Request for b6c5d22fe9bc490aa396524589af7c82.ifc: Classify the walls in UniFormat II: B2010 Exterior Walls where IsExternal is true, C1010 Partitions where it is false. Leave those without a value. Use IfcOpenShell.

First a look at what the model holds.

```python
import ifcopenshell
import ifcopenshell.util.element

model = ifcopenshell.open("b6c5d22fe9bc490aa396524589af7c82.ifc")
print(model.schema)
print("classifications:", [c.Name for c in model.by_type("IfcClassification")])
values = [ifcopenshell.util.element.get_pset(e, "Pset_WallCommon", "IsExternal") for e in model.by_type("IfcWall")]
for value in (True, False, None):
    print("IsExternal", value, values.count(value))
```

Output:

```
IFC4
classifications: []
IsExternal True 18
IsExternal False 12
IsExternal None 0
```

```python
import ifcopenshell
import ifcopenshell.api.classification
import ifcopenshell.util.element

model = ifcopenshell.open("b6c5d22fe9bc490aa396524589af7c82.ifc")

system = ifcopenshell.api.classification.add_classification(model, classification="UniFormat II")

walls = model.by_type("IfcWall")
external = {e: ifcopenshell.util.element.get_pset(e, "Pset_WallCommon", "IsExternal") for e in walls}
for flag, code, name in ((True, "B2010", "Exterior Walls"), (False, "C1010", "Partitions")):
    products = [e for e in walls if external[e] is flag]
    ifcopenshell.api.classification.add_reference(
        model, products=products, classification=system, identification=code, name=name
    )
    print(code, len(products))

model.write("b6c5d22fe9bc490aa396524589af7c82_rev.ifc")
```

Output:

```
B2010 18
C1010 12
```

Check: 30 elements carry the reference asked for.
